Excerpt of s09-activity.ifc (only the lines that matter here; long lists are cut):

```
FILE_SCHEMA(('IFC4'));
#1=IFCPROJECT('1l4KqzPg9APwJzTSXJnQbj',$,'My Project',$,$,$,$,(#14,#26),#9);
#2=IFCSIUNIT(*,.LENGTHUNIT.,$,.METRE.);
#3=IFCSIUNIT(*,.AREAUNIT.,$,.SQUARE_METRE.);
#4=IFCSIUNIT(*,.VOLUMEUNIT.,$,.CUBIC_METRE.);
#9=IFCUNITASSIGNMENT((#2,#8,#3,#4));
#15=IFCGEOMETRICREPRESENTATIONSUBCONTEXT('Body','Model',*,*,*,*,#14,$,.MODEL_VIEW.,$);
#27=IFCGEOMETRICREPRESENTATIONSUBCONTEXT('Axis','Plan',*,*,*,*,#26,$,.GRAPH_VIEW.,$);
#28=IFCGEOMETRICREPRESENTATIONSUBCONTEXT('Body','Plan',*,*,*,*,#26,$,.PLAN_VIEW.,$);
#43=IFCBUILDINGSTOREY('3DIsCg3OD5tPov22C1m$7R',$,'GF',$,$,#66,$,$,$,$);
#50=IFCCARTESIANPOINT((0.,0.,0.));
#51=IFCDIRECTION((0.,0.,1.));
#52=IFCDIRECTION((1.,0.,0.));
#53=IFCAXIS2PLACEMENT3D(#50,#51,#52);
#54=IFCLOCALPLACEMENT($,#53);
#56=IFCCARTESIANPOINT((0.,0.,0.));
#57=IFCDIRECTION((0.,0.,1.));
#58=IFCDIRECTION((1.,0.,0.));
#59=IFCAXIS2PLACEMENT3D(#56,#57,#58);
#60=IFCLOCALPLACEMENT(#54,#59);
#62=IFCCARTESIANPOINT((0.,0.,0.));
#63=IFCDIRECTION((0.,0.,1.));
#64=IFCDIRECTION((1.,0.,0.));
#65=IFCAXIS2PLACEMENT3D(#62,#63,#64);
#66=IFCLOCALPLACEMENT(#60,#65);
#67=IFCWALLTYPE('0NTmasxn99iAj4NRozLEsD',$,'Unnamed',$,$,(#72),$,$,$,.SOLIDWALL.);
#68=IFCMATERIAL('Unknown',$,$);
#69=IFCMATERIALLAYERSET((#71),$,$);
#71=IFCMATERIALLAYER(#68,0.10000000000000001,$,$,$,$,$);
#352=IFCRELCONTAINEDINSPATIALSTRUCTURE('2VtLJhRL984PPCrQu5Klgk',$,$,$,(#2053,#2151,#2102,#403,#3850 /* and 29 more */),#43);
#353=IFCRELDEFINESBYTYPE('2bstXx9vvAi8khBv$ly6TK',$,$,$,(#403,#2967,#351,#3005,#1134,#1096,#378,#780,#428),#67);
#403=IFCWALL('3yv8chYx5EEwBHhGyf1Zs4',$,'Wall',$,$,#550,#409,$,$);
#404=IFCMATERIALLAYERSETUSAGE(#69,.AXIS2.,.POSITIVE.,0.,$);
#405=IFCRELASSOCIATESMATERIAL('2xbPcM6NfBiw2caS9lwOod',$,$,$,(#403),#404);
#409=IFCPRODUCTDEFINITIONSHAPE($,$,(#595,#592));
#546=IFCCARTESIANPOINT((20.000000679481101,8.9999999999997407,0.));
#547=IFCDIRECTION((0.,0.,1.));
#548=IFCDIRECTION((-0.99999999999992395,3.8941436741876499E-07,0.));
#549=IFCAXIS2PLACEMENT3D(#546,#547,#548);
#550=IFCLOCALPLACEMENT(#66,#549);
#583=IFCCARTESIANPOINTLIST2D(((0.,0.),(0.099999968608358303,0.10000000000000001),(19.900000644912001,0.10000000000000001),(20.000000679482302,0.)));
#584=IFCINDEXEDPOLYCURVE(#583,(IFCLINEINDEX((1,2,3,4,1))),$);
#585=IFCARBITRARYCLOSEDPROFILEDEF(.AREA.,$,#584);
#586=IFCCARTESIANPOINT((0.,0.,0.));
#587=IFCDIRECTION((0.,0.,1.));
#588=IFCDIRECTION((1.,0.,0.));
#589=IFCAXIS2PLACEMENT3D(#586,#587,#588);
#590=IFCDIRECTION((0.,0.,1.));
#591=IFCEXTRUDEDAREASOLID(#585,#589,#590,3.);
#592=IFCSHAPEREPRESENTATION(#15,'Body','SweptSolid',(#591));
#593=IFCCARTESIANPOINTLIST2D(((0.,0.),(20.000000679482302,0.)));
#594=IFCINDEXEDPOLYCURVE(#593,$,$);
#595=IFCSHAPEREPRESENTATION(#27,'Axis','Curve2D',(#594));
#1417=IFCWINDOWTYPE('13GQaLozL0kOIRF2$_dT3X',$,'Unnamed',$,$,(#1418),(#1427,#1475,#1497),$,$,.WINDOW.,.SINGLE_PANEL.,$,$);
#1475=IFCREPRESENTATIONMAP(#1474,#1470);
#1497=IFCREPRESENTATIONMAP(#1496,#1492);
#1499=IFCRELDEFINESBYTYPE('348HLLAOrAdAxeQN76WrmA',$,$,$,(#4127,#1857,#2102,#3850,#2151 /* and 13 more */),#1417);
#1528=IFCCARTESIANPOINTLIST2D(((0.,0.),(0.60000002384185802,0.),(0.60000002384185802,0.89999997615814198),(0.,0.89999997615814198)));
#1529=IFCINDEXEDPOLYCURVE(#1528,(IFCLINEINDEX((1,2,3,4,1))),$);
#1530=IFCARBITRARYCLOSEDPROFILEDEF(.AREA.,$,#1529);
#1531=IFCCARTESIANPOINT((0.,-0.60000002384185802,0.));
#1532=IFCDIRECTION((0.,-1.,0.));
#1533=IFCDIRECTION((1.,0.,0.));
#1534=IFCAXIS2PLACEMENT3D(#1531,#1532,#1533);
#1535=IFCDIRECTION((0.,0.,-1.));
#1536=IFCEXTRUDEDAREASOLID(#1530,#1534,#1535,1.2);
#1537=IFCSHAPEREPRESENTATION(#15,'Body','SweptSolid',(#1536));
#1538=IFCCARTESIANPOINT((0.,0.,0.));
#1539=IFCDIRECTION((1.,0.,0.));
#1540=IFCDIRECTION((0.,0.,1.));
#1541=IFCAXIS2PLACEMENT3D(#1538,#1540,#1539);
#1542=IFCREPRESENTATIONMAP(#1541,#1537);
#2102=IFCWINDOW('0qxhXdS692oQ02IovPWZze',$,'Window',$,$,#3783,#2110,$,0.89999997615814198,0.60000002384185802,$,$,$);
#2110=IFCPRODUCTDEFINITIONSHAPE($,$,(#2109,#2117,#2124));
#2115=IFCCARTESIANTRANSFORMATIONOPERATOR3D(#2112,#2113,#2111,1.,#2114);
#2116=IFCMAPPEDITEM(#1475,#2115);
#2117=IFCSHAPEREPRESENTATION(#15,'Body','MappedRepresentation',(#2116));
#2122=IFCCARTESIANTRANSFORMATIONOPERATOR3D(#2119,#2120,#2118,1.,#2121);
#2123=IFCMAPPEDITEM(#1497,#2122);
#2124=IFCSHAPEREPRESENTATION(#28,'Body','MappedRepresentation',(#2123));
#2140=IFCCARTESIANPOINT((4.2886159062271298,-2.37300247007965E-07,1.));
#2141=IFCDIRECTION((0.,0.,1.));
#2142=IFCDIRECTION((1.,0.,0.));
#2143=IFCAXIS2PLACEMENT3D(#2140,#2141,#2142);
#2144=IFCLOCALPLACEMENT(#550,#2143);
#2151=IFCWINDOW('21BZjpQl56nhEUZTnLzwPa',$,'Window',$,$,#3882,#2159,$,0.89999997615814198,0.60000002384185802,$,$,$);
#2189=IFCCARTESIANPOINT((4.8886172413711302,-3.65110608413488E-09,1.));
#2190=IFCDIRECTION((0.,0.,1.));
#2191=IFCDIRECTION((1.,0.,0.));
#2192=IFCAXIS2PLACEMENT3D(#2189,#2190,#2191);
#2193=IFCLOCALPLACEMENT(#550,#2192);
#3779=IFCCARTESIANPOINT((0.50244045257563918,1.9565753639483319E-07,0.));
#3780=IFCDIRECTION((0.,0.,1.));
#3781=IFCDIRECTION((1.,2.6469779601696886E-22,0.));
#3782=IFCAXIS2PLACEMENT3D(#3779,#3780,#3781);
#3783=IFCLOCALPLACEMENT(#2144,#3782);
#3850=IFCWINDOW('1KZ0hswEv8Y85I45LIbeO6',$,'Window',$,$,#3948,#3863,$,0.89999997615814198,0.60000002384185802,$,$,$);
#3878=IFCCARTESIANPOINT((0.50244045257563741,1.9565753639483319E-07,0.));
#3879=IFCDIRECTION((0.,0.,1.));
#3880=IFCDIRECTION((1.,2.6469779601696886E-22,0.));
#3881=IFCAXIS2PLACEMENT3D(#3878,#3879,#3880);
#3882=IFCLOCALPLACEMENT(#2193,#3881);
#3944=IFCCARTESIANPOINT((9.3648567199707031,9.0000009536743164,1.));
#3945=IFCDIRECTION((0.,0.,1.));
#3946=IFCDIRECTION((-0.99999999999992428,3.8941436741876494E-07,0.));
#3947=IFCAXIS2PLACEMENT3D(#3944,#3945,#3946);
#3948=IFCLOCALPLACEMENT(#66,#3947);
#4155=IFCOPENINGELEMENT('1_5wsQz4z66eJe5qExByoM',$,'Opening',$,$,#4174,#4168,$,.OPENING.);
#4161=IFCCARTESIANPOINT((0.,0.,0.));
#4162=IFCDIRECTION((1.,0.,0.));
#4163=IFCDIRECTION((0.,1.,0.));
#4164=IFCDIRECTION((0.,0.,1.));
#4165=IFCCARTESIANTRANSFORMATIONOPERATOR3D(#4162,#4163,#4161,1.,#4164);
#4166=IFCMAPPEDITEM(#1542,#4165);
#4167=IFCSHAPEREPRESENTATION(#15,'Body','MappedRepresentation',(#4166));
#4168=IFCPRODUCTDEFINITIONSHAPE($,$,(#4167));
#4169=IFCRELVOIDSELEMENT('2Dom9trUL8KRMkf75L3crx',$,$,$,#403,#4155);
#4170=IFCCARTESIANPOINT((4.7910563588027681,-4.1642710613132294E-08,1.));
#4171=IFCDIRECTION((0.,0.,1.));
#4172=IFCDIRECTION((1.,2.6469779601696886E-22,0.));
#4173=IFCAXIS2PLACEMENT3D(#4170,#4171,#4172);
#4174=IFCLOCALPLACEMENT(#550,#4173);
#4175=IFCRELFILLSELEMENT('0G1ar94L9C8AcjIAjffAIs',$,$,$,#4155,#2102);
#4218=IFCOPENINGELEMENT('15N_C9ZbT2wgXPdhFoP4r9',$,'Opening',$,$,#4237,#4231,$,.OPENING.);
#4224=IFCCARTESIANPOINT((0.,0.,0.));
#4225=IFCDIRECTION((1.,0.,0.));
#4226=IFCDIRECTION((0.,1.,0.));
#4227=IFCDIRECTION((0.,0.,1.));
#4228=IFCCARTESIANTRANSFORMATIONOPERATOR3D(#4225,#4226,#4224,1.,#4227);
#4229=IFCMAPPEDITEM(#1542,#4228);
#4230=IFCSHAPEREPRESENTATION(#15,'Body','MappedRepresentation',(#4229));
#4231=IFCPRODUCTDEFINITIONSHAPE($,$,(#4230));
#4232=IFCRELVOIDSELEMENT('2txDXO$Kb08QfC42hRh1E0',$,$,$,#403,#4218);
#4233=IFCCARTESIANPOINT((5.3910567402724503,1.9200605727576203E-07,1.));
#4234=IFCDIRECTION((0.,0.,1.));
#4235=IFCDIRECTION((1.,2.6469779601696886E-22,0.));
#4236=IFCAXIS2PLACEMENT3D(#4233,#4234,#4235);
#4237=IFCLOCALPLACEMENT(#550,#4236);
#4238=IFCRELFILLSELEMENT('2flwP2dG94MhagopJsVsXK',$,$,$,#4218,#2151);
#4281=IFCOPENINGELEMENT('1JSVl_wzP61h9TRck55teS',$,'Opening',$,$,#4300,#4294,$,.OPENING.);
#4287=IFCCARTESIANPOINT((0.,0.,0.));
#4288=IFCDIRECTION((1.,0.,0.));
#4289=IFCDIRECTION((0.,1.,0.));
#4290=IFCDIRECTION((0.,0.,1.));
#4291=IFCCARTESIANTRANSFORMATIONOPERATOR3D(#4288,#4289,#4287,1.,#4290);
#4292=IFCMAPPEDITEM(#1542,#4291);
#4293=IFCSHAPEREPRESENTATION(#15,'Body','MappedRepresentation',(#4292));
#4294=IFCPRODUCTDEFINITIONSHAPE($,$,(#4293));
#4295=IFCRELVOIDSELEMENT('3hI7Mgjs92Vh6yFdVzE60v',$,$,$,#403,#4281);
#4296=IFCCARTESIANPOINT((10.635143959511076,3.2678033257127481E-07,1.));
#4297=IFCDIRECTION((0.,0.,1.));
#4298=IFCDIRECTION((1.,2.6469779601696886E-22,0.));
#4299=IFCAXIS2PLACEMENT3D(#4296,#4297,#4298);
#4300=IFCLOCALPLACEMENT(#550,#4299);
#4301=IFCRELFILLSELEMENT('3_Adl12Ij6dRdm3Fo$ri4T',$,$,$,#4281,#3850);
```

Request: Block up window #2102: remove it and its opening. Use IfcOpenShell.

```python
import ifcopenshell
import ifcopenshell.api.feature
import ifcopenshell.api.root
import ifcopenshell.geom
import ifcopenshell.util.shape

model = ifcopenshell.open("s09-activity.ifc")
settings = ifcopenshell.geom.settings()


def volume(element):
    """Net volume in cubic metres, openings subtracted."""
    shape = ifcopenshell.geom.create_shape(settings, element)
    return ifcopenshell.util.shape.get_volume(shape.geometry)


window = model.by_guid("0qxhXdS692oQ02IovPWZze")
opening = window.FillsVoids[0].RelatingOpeningElement
wall = opening.VoidsElements[0].RelatingBuildingElement
before = volume(wall)

ifcopenshell.api.root.remove_product(model, product=window)
ifcopenshell.api.feature.remove_feature(model, feature=opening)

after = volume(wall)

print(f"wall volume {before:.3f} -> {after:.3f} m3")

model.write("s09-activity-out.ifc")
```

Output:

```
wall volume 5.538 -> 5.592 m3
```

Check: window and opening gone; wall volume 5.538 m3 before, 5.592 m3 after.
